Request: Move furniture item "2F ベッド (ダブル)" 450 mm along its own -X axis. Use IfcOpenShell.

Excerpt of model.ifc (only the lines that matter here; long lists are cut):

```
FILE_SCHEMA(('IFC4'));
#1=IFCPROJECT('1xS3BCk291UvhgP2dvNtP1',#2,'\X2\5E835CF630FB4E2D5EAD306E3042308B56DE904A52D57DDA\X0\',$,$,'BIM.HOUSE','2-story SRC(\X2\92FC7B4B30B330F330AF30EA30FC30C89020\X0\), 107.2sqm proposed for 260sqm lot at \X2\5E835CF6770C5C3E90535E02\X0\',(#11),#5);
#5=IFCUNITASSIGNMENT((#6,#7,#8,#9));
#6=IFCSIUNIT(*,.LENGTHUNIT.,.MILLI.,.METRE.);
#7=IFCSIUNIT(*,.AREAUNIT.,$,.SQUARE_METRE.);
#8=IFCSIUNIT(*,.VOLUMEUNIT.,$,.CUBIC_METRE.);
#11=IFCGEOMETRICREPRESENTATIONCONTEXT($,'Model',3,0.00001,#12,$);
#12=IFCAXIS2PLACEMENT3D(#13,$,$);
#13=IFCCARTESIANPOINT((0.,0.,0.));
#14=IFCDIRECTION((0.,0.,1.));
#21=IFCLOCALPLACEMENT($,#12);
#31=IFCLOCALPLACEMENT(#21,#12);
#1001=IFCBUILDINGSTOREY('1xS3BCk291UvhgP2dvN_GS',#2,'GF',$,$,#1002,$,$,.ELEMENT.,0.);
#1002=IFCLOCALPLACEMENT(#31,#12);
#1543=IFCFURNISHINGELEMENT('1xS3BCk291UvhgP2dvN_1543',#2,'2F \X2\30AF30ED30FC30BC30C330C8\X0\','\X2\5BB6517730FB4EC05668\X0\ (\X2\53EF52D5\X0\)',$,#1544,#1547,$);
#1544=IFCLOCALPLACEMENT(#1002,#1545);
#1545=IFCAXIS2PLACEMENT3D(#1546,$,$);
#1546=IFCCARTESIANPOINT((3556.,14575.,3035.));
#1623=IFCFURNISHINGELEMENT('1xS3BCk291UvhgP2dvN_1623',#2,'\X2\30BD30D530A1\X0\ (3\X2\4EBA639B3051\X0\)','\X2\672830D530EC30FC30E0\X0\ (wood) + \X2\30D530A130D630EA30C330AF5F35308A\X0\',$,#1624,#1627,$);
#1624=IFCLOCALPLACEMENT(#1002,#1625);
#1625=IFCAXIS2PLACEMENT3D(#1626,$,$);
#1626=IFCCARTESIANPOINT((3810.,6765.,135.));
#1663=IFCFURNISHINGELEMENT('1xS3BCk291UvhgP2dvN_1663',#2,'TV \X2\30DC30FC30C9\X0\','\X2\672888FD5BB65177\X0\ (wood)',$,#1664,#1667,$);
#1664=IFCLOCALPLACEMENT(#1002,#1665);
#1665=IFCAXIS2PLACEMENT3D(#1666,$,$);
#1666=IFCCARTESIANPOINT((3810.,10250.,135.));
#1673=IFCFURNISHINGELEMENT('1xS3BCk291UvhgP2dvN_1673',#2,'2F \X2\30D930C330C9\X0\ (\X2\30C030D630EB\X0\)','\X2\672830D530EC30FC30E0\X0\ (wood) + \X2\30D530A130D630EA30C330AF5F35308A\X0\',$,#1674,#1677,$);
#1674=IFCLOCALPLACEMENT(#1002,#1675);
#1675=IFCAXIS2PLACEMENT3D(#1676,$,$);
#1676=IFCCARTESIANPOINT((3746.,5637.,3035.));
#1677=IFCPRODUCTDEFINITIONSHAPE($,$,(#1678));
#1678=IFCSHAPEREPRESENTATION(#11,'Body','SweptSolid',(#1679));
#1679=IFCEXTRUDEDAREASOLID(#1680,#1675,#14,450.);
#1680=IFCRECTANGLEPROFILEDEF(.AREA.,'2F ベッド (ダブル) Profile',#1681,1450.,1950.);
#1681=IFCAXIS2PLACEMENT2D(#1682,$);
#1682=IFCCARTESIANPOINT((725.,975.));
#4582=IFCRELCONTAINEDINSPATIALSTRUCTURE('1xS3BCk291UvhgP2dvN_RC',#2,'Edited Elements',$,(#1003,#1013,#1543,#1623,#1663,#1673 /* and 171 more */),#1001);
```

```python
import ifcopenshell
import ifcopenshell.api.geometry
import ifcopenshell.util.placement

model = ifcopenshell.open("model.ifc")

item = model.by_guid("1xS3BCk291UvhgP2dvN_1673")
matrix = ifcopenshell.util.placement.get_local_placement(item.ObjectPlacement)
matrix[:3, 3] -= matrix[:3, 0] * 450.0
ifcopenshell.api.geometry.edit_object_placement(model, product=item, matrix=matrix, is_si=False)

print(ifcopenshell.util.placement.get_local_placement(item.ObjectPlacement).round(3) + 0.0)

model.write("model_rev.ifc")
```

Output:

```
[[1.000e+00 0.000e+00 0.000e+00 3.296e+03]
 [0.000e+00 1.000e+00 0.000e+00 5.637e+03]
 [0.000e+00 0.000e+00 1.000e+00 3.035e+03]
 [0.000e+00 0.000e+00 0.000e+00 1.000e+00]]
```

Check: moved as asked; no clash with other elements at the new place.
